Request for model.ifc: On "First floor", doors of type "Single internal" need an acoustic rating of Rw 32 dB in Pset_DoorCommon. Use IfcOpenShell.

First a look at what the model holds.

```python
import ifcopenshell
import ifcopenshell.util.element

model = ifcopenshell.open("model.ifc")
print(model.schema)
storey = next(s for s in model.by_type("IfcBuildingStorey") if s.Name == "First floor")
doors = [e for e in ifcopenshell.util.element.get_decomposition(storey) if e.is_a("IfcDoor")]
seen = {}
for e in doors:
    element_type = ifcopenshell.util.element.get_type(e)
    key = (element_type.Name if element_type != e and element_type else None, ifcopenshell.util.element.get_pset(e, "Pset_DoorCommon", "AcousticRating"))
    seen[key] = seen.get(key, 0) + 1
for (name, value), count in sorted(seen.items(), key=str):
    print(count, "x", name, "|", value)
```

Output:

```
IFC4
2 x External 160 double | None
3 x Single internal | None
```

```python
import ifcopenshell
import ifcopenshell.api.pset
import ifcopenshell.util.element

model = ifcopenshell.open("model.ifc")

storey = next(s for s in model.by_type("IfcBuildingStorey") if s.Name == "First floor")
doors = [e for e in ifcopenshell.util.element.get_decomposition(storey) if e.is_a("IfcDoor")]

count = 0
for e in doors:
    element_type = ifcopenshell.util.element.get_type(e)
    if element_type in (None, e) or element_type.Name != "Single internal":
        continue
    # add_pset returns the element's existing set when there is one.
    pset = ifcopenshell.api.pset.add_pset(model, product=e, name="Pset_DoorCommon")
    ifcopenshell.api.pset.edit_pset(model, pset=pset, properties={"AcousticRating": "Rw 32 dB"})
    count += 1

print(count, "doors updated")

model.write("model-out.ifc")
```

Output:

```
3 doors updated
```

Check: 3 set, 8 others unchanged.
